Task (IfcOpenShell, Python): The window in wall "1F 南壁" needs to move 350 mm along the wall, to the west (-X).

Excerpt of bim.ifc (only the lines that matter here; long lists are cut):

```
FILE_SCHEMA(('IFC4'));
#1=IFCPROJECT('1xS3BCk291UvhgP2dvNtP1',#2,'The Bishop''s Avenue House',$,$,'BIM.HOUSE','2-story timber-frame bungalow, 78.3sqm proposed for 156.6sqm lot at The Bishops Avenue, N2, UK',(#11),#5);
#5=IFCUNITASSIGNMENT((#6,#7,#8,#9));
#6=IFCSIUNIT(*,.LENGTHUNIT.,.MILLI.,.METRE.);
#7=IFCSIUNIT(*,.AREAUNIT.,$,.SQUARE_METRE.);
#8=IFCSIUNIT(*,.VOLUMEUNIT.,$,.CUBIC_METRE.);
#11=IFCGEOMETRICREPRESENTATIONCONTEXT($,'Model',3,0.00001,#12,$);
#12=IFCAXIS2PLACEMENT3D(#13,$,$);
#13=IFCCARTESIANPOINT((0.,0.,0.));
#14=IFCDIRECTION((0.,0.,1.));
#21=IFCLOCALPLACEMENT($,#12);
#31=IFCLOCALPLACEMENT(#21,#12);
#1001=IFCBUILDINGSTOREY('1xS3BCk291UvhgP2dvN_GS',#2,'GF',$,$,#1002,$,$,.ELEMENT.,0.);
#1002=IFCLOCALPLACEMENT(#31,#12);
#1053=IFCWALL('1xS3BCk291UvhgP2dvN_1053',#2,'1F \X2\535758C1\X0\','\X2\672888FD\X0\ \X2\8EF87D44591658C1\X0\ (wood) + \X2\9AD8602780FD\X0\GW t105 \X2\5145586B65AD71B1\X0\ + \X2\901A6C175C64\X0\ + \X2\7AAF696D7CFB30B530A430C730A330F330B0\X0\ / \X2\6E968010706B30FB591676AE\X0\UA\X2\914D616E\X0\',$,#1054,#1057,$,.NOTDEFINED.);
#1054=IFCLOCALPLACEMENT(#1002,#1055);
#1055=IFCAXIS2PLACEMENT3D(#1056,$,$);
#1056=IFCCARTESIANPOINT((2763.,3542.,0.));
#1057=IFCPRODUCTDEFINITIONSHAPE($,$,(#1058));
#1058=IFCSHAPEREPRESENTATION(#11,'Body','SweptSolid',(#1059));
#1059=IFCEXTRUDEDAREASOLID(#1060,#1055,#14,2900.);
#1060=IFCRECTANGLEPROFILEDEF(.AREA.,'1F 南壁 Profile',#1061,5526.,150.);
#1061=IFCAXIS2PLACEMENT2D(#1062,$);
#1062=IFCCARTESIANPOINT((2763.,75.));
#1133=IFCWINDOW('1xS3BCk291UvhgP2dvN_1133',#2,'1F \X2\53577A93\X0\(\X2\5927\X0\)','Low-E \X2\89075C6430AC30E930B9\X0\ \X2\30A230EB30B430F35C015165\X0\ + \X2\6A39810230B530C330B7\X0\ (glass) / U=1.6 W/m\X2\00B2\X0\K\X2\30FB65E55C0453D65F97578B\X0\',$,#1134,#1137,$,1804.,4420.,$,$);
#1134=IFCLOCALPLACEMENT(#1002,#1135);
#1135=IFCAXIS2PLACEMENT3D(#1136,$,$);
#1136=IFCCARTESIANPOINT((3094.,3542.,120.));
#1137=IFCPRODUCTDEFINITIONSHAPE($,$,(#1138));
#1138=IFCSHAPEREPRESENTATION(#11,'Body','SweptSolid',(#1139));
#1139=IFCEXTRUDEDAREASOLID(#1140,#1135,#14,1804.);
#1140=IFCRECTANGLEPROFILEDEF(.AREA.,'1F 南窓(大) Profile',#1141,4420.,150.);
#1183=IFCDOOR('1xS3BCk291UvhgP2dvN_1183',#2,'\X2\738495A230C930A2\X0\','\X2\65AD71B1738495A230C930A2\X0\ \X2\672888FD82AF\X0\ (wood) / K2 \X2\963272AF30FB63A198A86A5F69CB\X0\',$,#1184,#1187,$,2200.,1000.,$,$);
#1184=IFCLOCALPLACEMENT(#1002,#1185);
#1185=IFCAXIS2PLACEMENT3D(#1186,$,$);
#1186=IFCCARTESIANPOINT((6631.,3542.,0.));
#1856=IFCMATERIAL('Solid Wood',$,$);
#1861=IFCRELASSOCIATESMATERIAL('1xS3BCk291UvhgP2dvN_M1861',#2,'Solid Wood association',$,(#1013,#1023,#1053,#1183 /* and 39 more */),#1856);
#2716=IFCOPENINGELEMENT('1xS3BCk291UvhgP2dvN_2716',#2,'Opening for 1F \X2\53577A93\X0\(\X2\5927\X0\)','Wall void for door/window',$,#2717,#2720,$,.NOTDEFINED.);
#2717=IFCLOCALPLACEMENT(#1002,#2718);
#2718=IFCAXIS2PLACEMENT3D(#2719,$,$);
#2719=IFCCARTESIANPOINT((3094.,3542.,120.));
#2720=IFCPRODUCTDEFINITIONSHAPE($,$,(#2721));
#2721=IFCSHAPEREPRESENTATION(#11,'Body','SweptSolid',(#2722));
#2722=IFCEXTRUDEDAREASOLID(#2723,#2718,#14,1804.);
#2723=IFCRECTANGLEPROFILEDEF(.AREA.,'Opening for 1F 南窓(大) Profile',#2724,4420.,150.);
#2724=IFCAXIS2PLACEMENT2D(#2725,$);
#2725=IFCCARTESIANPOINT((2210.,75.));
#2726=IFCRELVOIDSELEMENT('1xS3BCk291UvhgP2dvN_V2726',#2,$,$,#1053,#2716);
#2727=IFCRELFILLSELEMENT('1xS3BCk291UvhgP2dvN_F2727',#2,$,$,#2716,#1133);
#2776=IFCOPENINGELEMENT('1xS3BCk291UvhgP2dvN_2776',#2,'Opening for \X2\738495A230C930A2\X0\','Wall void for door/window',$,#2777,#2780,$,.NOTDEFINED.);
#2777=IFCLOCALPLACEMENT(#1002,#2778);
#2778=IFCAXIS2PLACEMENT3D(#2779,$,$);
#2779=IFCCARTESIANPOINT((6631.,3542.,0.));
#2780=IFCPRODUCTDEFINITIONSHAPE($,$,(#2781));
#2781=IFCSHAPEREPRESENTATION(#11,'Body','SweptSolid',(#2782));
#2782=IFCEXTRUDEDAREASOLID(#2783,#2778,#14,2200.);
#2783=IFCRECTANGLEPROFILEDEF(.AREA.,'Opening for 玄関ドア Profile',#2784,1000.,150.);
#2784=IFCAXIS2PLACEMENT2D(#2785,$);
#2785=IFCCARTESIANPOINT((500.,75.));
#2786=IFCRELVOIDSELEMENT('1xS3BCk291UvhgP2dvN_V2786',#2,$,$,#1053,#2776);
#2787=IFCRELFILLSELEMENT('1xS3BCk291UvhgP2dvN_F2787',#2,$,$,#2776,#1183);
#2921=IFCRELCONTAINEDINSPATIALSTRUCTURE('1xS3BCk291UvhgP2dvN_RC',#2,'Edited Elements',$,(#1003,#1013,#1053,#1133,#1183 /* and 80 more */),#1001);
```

```python
import ifcopenshell
import ifcopenshell.api.geometry
import ifcopenshell.util.placement

model = ifcopenshell.open("bim.ifc")

window = model.by_guid("1xS3BCk291UvhgP2dvN_1133")
opening = window.FillsVoids[0].RelatingOpeningElement
wall = opening.VoidsElements[0].RelatingBuildingElement

wall_matrix = ifcopenshell.util.placement.get_local_placement(wall.ObjectPlacement)
shift = wall_matrix[:3, 0] * -350.0
before = ifcopenshell.util.placement.get_local_placement(window.ObjectPlacement)[:3, 3].copy()

# The window is not placed relative to its opening, so move both.
for product in (opening, window):
    matrix = ifcopenshell.util.placement.get_local_placement(product.ObjectPlacement)
    matrix[:3, 3] += shift
    ifcopenshell.api.geometry.edit_object_placement(model, product=product, matrix=matrix, is_si=False)

after = ifcopenshell.util.placement.get_local_placement(window.ObjectPlacement)[:3, 3]
print("window moved by", (after - before).round(3) + 0.0)

model.write("bim-out.ifc")
```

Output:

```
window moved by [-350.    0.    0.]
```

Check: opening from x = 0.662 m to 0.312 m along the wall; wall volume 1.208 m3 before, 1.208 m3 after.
